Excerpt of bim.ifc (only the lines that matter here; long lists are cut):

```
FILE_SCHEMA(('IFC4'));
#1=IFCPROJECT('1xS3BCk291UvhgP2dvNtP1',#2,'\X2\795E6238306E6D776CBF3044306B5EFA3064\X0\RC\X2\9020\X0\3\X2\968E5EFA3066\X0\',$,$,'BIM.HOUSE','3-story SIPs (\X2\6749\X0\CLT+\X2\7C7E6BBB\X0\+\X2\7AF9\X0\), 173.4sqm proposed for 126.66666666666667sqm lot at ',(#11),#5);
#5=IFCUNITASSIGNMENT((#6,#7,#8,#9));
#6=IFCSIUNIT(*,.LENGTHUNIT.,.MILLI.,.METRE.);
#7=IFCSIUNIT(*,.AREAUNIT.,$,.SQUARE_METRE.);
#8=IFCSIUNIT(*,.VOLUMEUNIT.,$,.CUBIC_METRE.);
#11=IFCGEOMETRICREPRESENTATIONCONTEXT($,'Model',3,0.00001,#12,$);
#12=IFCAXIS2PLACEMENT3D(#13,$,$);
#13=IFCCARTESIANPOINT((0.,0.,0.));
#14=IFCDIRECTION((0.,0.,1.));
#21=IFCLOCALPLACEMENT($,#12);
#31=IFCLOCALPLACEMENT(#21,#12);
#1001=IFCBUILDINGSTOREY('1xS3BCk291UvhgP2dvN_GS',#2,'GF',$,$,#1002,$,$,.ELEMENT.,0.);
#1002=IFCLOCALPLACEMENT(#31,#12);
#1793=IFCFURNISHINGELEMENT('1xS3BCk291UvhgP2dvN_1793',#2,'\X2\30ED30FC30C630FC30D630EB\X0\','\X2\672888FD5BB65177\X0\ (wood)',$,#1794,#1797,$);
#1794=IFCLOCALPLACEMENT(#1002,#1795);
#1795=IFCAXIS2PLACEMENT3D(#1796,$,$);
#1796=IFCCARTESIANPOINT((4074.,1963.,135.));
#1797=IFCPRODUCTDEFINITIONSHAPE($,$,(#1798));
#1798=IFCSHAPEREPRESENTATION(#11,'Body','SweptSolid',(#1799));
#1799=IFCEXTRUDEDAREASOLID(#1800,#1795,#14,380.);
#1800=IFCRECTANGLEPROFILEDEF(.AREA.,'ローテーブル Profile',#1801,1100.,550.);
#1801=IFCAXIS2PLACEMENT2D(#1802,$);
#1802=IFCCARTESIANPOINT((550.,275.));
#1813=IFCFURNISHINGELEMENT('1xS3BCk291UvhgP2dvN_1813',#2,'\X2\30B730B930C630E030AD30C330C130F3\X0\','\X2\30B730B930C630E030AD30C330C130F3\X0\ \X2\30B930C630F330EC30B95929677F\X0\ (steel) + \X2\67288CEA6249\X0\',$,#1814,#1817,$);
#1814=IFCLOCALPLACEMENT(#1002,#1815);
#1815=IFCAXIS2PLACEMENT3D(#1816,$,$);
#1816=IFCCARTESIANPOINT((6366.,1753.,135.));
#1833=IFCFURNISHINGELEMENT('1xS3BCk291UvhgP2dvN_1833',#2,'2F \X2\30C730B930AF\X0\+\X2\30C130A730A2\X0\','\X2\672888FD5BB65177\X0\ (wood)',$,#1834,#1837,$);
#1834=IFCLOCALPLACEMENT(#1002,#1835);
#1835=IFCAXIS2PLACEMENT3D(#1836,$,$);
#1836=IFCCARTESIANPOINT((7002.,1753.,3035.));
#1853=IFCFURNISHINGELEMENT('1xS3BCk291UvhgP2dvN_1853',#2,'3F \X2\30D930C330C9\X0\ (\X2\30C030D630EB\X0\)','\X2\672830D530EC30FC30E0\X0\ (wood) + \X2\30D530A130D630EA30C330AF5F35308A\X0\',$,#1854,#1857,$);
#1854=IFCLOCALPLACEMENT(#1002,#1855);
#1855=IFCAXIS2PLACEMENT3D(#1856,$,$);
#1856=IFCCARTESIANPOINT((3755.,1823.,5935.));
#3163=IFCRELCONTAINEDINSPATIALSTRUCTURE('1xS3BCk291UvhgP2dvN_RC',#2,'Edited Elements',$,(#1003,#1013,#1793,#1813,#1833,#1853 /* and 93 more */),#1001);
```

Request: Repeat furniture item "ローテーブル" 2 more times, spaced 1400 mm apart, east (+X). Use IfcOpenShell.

```python
import numpy as np
import ifcopenshell
import ifcopenshell.api.geometry
import ifcopenshell.api.root
import ifcopenshell.util.element
import ifcopenshell.util.placement
import ifcopenshell.util.unit

model = ifcopenshell.open("bim.ifc")
unit_scale = ifcopenshell.util.unit.calculate_unit_scale(model)


def reuse_history(source, copy):
    """copy_class also copies each property set's owner history, people and application; keep the originals."""
    for rel in copy.IsDefinedBy:
        if rel.is_a("IfcRelDefinesByProperties") and (history := rel.RelatingPropertyDefinition.OwnerHistory):
            rel.RelatingPropertyDefinition.OwnerHistory = source.OwnerHistory
            ifcopenshell.util.element.remove_deep2(model, history)


source = model.by_id(1793)
base = ifcopenshell.util.placement.get_local_placement(source.ObjectPlacement)
step = np.array([1.0, 0.0, 0.0]) * 1.4 / unit_scale

for i in range(1, 3):
    copy = ifcopenshell.api.root.copy_class(model, product=source)
    copy.Representation = ifcopenshell.util.element.copy_deep(
        model, source.Representation, exclude=["IfcGeometricRepresentationContext", "IfcRepresentationMap"]
    )
    reuse_history(source, copy)
    matrix = base.copy()
    matrix[:3, 3] += i * step
    print("added at", matrix[:3, 3].round(3) + 0.0)
    ifcopenshell.api.geometry.edit_object_placement(model, product=copy, matrix=matrix, is_si=False)

model.write("bim_v2.ifc")
```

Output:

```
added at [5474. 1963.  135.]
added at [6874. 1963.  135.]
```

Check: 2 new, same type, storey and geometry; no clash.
